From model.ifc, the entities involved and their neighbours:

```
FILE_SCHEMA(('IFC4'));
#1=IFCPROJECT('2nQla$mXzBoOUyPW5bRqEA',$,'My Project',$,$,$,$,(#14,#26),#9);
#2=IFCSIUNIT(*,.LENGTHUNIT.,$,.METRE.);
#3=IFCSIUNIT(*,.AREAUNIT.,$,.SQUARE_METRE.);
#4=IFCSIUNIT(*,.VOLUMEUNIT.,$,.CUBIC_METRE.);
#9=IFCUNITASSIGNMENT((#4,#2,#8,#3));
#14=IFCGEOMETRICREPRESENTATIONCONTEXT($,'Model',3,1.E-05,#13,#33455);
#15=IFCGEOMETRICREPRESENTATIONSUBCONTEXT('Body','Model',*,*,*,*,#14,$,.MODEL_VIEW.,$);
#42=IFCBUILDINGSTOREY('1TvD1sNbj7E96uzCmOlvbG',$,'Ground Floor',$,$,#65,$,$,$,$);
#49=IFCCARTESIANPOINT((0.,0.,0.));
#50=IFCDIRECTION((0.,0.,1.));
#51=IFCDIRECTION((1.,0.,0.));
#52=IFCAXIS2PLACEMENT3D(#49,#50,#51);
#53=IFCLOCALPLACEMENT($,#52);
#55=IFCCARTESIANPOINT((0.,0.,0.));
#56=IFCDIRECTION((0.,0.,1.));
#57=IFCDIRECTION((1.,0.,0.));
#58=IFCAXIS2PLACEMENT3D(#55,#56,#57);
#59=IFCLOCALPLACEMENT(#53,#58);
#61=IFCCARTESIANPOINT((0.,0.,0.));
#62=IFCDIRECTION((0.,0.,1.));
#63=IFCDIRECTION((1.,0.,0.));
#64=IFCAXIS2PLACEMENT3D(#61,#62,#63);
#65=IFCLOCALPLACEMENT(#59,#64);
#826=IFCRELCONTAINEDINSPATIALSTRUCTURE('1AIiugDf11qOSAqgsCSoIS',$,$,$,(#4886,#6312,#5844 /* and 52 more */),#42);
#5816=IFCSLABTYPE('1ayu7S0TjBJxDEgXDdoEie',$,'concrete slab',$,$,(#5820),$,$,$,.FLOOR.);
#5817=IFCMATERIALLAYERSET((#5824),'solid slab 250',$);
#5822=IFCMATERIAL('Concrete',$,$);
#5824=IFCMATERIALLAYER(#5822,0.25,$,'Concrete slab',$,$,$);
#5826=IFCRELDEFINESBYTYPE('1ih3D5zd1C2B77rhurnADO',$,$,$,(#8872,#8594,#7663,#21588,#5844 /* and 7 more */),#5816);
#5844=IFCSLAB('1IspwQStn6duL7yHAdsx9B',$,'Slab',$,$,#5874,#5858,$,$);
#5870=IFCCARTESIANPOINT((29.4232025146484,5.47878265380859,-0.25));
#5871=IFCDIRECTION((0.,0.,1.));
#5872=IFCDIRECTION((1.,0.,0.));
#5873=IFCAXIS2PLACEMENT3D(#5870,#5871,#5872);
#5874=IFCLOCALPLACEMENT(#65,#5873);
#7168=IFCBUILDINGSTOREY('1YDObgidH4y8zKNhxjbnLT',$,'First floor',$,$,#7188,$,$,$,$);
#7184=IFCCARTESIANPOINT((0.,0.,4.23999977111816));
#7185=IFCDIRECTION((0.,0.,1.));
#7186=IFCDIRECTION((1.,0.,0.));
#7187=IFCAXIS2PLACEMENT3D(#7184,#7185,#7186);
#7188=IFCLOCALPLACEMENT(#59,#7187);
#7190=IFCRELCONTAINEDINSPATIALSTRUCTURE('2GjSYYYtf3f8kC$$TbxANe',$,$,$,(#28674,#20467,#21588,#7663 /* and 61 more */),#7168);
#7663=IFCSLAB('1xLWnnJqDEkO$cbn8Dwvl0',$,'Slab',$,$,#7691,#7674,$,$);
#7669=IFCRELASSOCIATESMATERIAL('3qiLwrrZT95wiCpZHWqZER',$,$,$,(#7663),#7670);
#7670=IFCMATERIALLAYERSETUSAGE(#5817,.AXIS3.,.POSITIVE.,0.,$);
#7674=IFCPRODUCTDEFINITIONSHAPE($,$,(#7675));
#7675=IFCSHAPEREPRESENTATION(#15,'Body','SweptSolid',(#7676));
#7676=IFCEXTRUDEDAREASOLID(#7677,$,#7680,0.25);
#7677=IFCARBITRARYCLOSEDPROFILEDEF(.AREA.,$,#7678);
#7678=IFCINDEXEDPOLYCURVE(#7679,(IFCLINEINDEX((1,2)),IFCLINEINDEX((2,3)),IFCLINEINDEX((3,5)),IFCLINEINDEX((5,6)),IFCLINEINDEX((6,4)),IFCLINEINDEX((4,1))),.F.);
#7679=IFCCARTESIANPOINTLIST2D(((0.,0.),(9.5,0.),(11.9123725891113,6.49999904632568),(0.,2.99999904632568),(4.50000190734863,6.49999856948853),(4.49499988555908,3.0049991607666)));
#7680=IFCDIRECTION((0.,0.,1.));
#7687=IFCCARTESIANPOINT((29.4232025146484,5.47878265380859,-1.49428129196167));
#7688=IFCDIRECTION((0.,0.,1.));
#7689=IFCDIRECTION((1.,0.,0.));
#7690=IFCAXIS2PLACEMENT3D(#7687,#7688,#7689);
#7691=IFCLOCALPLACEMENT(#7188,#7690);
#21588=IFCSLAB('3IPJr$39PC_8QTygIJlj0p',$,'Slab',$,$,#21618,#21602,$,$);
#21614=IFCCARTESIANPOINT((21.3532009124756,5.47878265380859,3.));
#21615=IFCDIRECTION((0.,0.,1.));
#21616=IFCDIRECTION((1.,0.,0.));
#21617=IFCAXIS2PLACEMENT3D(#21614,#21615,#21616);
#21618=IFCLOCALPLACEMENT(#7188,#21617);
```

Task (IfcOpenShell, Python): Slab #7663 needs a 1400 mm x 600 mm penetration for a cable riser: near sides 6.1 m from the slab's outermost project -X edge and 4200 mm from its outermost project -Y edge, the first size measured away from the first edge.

```python
import numpy as np
import ifcopenshell
import ifcopenshell.api.feature
import ifcopenshell.api.geometry
import ifcopenshell.api.root
import ifcopenshell.geom
import ifcopenshell.util.placement
import ifcopenshell.util.representation
import ifcopenshell.util.shape
import ifcopenshell.util.unit

model = ifcopenshell.open("model.ifc")
unit_scale = ifcopenshell.util.unit.calculate_unit_scale(model)
settings = ifcopenshell.geom.settings()


def volume(element):
    """Net volume in cubic metres, openings subtracted."""
    shape = ifcopenshell.geom.create_shape(settings, element)
    return ifcopenshell.util.shape.get_volume(shape.geometry)


slab = model.by_guid("1xLWnnJqDEkO$cbn8Dwvl0")
before = volume(slab)

# Extent in the slab's own axes, in metres. The edges named are its -X and -Y sides.
slab_shape = ifcopenshell.geom.create_shape(settings, slab)
vertices = ifcopenshell.util.shape.get_vertices(slab_shape.geometry)
x_min, y_min, bottom = vertices.min(axis=0)
top = vertices[:, 2].max()

opening = ifcopenshell.api.root.create_entity(model, ifc_class="IfcOpeningElement", name="Cable riser opening", predefined_type="OPENING")
context = ifcopenshell.util.representation.get_context(model, "Model", "Body", "MODEL_VIEW")
width, depth = 1.4, 0.6
outline = [(0.0, 0.0), (width, 0.0), (width, depth), (0.0, depth), (0.0, 0.0)]
# Overshoot both faces by 50 mm so the cut is clean.
shape = ifcopenshell.api.geometry.add_slab_representation(
    model, context=context, depth=top - bottom + 0.1, polyline=outline
)
ifcopenshell.api.geometry.assign_representation(model, product=opening, representation=shape)

matrix = ifcopenshell.util.placement.get_local_placement(slab.ObjectPlacement)
matrix[:, 3] = matrix @ np.append(np.array([x_min + 6.1, y_min + 4.2, bottom - 0.05]) / unit_scale, 1.0)
ifcopenshell.api.geometry.edit_object_placement(model, product=opening, matrix=matrix, is_si=False)
ifcopenshell.api.feature.add_feature(model, feature=opening, element=slab)

after = volume(slab)

print(f"slab volume {before:.3f} -> {after:.3f} m3")

model.write("model-out.ifc")
```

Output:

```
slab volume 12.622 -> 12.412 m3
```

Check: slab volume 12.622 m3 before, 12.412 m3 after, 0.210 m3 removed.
